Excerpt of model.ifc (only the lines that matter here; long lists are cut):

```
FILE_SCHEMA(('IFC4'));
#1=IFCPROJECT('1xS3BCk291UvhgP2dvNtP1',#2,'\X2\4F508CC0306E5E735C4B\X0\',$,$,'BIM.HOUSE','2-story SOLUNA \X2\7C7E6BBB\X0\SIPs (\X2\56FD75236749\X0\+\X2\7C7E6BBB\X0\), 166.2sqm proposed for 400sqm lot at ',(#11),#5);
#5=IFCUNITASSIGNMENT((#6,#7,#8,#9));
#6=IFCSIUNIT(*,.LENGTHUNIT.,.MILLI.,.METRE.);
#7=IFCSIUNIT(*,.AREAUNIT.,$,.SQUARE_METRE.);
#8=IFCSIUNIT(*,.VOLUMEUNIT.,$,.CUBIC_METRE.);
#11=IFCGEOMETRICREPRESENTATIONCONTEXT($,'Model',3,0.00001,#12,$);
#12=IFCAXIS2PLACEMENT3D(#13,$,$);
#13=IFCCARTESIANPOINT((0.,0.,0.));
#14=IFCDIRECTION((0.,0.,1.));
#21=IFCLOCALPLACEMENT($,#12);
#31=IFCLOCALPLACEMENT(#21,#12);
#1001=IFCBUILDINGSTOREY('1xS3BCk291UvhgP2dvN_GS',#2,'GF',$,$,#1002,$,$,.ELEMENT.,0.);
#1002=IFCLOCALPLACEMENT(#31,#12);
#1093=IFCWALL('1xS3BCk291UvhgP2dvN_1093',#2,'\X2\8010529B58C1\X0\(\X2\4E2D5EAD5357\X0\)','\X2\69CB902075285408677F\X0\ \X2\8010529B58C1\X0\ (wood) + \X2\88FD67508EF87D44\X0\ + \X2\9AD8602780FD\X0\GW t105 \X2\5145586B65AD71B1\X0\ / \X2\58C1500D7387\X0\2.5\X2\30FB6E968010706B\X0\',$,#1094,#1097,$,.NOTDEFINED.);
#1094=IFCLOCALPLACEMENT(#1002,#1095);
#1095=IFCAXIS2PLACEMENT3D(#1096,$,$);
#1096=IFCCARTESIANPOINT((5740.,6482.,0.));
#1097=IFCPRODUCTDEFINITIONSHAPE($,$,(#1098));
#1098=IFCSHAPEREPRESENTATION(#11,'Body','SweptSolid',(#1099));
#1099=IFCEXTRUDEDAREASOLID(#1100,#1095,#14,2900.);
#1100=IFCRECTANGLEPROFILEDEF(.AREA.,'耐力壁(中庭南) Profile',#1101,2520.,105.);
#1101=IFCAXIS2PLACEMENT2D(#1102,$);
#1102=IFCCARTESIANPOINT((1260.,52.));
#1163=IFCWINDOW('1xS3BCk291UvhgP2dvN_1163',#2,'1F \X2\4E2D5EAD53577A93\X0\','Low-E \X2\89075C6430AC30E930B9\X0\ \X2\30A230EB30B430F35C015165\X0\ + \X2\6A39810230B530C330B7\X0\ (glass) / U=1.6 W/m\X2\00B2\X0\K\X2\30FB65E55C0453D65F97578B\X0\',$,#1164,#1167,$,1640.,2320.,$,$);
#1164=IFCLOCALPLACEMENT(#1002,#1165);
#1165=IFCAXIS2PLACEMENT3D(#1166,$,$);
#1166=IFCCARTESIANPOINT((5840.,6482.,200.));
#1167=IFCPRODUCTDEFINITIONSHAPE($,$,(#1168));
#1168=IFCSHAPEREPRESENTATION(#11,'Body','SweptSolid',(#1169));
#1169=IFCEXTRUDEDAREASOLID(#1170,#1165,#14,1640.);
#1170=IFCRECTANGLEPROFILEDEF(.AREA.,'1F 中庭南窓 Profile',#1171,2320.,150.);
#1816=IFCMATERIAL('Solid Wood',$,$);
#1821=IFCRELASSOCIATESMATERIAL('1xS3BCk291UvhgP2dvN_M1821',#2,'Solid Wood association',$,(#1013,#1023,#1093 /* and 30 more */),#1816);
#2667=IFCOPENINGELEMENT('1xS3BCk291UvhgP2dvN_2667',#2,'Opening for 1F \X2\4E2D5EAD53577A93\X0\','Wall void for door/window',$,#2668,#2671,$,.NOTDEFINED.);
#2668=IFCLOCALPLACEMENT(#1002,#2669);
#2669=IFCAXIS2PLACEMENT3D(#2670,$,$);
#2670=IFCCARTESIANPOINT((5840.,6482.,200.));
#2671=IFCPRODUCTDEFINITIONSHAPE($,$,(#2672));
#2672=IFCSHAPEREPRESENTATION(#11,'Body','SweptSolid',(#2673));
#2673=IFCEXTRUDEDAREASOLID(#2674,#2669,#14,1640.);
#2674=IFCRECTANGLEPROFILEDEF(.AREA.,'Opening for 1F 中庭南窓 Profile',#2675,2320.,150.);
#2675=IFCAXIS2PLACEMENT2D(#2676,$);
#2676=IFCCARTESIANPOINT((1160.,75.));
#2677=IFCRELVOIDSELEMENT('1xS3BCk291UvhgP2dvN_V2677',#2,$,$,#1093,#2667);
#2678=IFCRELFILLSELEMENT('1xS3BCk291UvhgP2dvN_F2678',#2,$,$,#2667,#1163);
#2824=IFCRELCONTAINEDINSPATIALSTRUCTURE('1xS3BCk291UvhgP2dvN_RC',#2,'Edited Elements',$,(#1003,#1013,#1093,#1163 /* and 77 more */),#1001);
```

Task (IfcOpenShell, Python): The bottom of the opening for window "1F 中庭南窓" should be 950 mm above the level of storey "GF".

```python
import numpy as np
import ifcopenshell
import ifcopenshell.api.geometry
import ifcopenshell.geom
import ifcopenshell.util.element
import ifcopenshell.util.placement
import ifcopenshell.util.shape
import ifcopenshell.util.unit

model = ifcopenshell.open("model.ifc")
unit_scale = ifcopenshell.util.unit.calculate_unit_scale(model)

window = model.by_id(1163)
opening = window.FillsVoids[0].RelatingOpeningElement
storey = ifcopenshell.util.element.get_container(window, ifc_class="IfcBuildingStorey")
level = ifcopenshell.util.placement.get_local_placement(storey.ObjectPlacement)[2, 3]

# The opening's origin need not be at the sill, so measure its lowest point.
shape = ifcopenshell.geom.create_shape(ifcopenshell.geom.settings(), opening)
bottom = ifcopenshell.util.shape.get_shape_bottom_elevation(shape, shape.geometry) / unit_scale
dz = level + 950.0 - bottom

shift = np.array([0.0, 0.0, dz])
# The window is not placed relative to its opening, so move both.
for product in (opening, window):
    matrix = ifcopenshell.util.placement.get_local_placement(product.ObjectPlacement)
    matrix[:3, 3] += shift
    ifcopenshell.api.geometry.edit_object_placement(model, product=product, matrix=matrix, is_si=False)

print(f"moved by {dz * unit_scale:+.3f} m")

model.write("model_v2.ifc")
```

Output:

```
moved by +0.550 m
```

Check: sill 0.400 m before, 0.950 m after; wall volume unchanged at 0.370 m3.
